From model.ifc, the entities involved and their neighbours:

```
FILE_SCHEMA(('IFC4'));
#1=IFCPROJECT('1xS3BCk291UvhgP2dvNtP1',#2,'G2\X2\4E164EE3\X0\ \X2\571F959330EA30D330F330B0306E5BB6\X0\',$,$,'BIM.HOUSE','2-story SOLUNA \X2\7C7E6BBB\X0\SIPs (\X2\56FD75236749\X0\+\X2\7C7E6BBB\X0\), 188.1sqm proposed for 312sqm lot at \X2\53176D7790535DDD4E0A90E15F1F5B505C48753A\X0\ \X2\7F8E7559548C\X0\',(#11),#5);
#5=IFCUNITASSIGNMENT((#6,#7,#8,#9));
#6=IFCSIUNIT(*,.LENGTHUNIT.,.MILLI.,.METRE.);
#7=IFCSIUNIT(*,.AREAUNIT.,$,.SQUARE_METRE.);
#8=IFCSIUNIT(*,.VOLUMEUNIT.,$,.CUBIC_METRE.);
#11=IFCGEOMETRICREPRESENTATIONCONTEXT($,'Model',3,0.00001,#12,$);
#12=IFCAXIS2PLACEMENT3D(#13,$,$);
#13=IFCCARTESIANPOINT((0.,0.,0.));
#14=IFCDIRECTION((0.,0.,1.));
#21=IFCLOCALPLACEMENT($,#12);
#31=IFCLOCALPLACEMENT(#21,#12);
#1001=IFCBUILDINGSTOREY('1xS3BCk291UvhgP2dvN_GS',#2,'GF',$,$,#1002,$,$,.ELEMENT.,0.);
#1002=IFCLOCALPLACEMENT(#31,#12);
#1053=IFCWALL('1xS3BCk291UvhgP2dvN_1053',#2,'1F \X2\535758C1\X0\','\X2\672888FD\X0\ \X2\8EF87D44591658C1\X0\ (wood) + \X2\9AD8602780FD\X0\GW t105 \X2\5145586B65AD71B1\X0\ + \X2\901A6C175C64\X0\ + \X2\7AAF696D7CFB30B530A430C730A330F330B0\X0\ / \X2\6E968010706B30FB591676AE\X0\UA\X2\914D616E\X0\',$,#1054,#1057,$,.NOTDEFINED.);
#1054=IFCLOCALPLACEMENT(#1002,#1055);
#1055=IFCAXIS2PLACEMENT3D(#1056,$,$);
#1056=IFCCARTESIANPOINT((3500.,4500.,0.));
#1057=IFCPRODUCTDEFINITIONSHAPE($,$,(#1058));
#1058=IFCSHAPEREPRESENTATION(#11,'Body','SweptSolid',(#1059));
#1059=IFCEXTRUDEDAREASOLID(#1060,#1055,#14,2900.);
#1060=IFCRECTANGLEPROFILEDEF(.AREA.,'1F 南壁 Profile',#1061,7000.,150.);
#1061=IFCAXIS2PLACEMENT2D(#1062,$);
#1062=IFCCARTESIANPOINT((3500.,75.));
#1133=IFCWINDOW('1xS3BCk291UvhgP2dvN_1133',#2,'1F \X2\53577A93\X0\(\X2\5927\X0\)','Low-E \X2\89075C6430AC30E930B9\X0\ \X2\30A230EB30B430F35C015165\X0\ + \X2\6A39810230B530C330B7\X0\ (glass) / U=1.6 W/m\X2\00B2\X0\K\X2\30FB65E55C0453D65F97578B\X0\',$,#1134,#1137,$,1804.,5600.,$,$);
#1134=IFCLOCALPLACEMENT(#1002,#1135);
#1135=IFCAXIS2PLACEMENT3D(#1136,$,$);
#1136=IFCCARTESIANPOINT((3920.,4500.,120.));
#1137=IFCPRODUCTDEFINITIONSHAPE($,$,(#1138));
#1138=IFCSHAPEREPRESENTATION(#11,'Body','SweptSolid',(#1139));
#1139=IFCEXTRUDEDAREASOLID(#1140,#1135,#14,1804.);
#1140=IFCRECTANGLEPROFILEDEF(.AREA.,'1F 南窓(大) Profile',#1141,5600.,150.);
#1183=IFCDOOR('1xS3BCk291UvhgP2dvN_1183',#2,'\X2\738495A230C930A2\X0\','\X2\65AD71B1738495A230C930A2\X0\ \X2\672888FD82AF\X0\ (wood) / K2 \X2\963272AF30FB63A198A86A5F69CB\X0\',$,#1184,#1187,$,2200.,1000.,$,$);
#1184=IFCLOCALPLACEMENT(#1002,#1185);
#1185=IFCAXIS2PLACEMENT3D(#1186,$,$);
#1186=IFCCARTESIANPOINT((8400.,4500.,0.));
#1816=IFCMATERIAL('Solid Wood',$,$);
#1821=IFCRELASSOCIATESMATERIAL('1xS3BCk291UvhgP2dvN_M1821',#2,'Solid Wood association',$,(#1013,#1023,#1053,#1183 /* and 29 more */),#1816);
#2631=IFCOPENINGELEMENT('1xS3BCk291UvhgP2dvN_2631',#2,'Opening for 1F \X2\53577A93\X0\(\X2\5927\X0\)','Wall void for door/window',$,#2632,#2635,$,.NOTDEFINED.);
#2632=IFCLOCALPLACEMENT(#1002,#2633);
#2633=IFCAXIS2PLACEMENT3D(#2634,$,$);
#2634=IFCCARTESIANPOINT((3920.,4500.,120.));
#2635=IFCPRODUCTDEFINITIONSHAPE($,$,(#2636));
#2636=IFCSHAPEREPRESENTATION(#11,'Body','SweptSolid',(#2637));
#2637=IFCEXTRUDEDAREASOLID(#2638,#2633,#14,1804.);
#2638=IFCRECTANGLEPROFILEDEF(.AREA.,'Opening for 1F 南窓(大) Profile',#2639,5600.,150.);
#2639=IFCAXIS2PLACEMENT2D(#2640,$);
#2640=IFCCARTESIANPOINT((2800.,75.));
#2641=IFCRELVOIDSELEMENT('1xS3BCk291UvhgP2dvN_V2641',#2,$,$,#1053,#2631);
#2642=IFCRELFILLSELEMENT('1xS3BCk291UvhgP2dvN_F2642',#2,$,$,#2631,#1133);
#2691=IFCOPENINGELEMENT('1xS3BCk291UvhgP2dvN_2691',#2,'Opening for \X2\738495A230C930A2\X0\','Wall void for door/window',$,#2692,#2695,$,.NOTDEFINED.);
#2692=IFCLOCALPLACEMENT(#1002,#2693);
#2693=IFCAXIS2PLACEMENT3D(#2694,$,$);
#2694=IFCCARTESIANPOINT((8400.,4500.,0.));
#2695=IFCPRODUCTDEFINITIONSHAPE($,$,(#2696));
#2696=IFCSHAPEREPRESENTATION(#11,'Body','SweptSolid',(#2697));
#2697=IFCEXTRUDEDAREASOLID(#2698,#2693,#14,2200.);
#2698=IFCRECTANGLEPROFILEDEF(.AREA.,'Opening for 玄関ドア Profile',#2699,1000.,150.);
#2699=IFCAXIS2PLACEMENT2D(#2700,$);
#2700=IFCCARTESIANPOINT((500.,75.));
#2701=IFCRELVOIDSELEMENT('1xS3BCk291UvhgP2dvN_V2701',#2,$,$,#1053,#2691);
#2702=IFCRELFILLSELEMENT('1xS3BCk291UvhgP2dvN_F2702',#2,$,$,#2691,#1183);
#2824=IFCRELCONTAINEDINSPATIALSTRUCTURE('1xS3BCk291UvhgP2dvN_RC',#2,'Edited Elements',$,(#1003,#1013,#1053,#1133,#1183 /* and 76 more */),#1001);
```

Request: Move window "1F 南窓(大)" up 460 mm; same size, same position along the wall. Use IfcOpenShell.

```python
import numpy as np
import ifcopenshell
import ifcopenshell.api.geometry
import ifcopenshell.util.placement
import ifcopenshell.util.unit

model = ifcopenshell.open("model.ifc")
unit_scale = ifcopenshell.util.unit.calculate_unit_scale(model)

window = model.by_guid("1xS3BCk291UvhgP2dvN_1133")
opening = window.FillsVoids[0].RelatingOpeningElement
dz = 460.0

shift = np.array([0.0, 0.0, dz])
# The window is not placed relative to its opening, so move both.
for product in (opening, window):
    matrix = ifcopenshell.util.placement.get_local_placement(product.ObjectPlacement)
    matrix[:3, 3] += shift
    ifcopenshell.api.geometry.edit_object_placement(model, product=product, matrix=matrix, is_si=False)

print(f"moved by {dz * unit_scale:+.3f} m")

model.write("model_updated.ifc")
```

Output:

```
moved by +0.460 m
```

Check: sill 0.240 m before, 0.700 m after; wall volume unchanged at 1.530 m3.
